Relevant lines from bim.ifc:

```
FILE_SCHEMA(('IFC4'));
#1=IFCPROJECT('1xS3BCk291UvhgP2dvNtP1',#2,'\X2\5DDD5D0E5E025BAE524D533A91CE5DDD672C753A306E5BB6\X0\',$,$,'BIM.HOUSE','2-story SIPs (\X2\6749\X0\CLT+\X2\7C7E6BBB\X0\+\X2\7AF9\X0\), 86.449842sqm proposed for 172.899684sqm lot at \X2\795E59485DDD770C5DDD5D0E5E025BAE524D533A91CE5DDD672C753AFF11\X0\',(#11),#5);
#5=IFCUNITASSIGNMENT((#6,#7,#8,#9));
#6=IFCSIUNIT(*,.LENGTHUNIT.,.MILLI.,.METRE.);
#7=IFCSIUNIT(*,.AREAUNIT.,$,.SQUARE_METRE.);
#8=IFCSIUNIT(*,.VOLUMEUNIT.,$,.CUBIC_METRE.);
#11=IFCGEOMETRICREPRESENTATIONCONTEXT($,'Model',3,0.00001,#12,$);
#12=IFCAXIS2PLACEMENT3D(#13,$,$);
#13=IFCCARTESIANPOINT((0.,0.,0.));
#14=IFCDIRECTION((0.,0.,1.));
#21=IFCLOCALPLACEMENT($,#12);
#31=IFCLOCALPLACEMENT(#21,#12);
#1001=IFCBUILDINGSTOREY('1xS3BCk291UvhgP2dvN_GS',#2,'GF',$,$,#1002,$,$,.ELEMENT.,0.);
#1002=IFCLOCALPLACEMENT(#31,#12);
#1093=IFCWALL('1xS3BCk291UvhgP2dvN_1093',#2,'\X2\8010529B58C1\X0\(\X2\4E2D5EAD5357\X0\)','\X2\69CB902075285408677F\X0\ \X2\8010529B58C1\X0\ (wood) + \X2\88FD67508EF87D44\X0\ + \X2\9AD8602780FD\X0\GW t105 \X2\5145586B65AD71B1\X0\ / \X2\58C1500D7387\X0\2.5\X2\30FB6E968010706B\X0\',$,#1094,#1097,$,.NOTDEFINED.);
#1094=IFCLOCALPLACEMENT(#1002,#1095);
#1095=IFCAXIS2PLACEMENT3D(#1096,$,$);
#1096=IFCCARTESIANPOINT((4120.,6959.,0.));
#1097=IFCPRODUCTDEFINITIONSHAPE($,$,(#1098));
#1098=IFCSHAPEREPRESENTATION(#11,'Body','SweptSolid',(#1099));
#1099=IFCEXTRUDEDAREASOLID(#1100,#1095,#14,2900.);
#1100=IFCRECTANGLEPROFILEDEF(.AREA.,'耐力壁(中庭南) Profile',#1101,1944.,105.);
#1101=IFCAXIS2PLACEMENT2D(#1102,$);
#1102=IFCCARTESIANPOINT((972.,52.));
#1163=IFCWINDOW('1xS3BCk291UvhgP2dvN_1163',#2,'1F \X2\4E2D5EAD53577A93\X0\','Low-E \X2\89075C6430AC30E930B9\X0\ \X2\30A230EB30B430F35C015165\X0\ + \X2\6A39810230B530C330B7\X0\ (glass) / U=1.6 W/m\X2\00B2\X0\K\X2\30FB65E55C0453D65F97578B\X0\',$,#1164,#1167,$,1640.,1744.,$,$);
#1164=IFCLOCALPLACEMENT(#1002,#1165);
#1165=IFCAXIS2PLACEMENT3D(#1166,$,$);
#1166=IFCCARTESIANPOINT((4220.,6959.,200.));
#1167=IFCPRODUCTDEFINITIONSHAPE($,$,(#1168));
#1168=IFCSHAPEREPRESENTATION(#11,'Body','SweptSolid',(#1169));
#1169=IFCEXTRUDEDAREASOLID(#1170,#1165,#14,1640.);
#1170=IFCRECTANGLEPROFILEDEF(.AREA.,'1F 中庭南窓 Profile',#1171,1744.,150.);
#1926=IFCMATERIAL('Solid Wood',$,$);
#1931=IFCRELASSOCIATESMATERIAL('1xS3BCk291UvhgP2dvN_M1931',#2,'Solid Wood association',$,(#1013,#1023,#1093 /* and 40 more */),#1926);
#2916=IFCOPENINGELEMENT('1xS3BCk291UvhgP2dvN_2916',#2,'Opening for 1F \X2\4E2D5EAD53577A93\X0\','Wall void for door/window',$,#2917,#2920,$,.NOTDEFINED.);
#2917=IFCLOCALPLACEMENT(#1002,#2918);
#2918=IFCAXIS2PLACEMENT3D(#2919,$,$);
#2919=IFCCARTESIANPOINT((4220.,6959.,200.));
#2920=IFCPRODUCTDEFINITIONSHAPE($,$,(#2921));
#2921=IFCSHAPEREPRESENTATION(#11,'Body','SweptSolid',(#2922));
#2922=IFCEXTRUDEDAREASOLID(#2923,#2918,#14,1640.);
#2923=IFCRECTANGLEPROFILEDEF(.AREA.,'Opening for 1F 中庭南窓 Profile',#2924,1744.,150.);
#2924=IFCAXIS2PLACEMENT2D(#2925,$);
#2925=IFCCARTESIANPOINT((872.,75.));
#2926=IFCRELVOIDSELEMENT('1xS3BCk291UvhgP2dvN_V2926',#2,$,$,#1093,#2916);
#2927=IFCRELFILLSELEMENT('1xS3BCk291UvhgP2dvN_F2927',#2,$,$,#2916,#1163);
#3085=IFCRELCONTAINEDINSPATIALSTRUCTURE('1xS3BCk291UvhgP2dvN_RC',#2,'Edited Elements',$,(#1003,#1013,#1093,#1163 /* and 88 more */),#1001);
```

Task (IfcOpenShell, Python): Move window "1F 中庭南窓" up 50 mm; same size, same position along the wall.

```python
import numpy as np
import ifcopenshell
import ifcopenshell.api.geometry
import ifcopenshell.util.placement
import ifcopenshell.util.unit

model = ifcopenshell.open("bim.ifc")
unit_scale = ifcopenshell.util.unit.calculate_unit_scale(model)

window = model.by_guid("1xS3BCk291UvhgP2dvN_1163")
opening = window.FillsVoids[0].RelatingOpeningElement
dz = 50.0

shift = np.array([0.0, 0.0, dz])
# The window is not placed relative to its opening, so move both.
for product in (opening, window):
    matrix = ifcopenshell.util.placement.get_local_placement(product.ObjectPlacement)
    matrix[:3, 3] += shift
    ifcopenshell.api.geometry.edit_object_placement(model, product=product, matrix=matrix, is_si=False)

print(f"moved by {dz * unit_scale:+.3f} m")

model.write("bim_updated.ifc")
```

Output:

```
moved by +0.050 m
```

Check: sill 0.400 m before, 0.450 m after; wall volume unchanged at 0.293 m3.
